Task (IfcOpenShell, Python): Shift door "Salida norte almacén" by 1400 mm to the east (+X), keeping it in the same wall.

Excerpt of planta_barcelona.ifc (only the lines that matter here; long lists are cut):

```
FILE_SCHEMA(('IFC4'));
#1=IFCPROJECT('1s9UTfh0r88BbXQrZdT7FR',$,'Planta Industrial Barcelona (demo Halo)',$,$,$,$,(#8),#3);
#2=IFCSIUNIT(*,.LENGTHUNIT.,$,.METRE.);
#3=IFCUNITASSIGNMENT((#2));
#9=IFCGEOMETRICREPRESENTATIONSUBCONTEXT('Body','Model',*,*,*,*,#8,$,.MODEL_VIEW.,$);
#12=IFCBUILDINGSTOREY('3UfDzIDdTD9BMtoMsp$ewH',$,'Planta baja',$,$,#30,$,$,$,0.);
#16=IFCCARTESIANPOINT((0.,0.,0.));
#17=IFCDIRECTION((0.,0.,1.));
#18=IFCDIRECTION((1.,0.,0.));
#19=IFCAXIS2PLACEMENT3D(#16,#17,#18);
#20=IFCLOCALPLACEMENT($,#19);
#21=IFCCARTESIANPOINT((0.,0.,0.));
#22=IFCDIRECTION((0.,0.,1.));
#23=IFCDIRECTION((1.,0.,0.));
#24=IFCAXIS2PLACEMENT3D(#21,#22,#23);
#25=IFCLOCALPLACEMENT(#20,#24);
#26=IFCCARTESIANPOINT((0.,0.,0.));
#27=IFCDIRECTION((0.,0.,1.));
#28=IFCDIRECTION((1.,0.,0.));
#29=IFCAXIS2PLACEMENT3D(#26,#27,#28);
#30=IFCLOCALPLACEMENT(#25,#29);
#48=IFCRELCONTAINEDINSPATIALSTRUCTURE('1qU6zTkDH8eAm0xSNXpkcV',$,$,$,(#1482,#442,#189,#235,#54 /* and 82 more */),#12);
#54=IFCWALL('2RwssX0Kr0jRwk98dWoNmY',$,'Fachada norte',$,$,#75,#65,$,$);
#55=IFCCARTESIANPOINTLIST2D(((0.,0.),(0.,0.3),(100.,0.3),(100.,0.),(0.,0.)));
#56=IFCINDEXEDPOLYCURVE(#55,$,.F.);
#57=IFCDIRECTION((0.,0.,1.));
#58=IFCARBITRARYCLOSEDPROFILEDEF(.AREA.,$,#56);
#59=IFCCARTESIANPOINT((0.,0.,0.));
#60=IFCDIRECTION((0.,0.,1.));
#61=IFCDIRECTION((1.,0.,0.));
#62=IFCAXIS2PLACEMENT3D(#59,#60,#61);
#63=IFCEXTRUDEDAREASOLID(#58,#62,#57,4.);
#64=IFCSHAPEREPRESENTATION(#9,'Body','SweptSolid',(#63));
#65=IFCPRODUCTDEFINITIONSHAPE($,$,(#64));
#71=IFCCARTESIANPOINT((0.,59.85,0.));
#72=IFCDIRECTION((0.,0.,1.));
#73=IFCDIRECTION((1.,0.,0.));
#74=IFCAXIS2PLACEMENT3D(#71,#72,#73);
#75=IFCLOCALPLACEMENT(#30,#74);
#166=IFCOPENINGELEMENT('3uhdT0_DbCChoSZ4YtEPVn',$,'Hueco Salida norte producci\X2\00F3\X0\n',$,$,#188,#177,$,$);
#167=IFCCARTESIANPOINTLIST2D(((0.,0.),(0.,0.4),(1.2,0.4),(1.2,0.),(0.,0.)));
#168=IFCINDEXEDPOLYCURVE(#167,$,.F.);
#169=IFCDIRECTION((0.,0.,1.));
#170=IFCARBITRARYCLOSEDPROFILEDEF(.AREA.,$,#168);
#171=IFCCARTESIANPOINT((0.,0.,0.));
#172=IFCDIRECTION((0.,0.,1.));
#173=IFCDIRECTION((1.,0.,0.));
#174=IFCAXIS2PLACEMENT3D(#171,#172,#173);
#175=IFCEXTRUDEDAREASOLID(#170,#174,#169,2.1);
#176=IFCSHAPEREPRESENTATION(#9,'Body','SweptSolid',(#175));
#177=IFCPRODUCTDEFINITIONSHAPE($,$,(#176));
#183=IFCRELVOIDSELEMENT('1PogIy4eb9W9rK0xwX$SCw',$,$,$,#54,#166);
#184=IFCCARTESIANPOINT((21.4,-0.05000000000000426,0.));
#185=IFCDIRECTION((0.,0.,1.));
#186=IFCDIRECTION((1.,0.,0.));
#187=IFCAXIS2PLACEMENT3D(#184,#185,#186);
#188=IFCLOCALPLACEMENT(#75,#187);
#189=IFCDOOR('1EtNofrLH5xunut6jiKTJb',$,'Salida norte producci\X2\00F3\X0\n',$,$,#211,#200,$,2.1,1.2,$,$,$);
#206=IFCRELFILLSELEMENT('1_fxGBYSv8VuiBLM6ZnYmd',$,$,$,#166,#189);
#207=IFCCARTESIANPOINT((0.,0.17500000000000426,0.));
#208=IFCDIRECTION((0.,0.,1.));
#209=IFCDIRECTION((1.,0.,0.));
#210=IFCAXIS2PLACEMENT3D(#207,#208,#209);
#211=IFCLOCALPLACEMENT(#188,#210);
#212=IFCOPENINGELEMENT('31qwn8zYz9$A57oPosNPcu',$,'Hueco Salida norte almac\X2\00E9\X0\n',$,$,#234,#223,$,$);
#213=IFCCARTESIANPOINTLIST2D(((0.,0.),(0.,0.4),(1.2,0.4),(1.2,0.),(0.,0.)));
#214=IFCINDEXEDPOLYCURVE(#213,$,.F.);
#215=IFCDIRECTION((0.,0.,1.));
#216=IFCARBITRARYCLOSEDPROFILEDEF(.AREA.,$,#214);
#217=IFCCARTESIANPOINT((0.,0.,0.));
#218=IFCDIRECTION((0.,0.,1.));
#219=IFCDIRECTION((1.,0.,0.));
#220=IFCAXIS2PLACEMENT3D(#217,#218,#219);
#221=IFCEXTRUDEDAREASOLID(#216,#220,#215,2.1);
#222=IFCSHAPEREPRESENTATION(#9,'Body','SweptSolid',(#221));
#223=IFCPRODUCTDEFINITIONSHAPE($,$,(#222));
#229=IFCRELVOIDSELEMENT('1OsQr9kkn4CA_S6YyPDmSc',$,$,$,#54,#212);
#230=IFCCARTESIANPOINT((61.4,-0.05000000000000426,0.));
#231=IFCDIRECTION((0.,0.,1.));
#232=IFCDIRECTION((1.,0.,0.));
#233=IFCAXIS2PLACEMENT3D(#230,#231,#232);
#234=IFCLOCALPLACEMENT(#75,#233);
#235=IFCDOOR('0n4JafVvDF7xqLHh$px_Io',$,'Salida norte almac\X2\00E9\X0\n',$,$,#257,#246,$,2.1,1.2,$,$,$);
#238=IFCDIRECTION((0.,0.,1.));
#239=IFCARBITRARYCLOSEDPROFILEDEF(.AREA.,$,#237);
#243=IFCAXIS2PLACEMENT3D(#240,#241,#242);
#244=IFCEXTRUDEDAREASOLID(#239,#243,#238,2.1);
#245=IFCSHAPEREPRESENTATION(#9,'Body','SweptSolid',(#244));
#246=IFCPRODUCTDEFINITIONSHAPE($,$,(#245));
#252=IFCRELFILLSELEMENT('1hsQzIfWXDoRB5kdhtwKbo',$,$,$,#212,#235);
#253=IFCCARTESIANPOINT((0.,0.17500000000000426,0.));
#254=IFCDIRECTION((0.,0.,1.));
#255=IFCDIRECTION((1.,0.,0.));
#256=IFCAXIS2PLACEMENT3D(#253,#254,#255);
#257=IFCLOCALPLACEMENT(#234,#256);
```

```python
import ifcopenshell
import ifcopenshell.api.geometry
import ifcopenshell.util.placement
import ifcopenshell.util.unit

model = ifcopenshell.open("planta_barcelona.ifc")
unit_scale = ifcopenshell.util.unit.calculate_unit_scale(model)

door = model.by_guid("0n4JafVvDF7xqLHh$px_Io")
opening = door.FillsVoids[0].RelatingOpeningElement
wall = opening.VoidsElements[0].RelatingBuildingElement

wall_matrix = ifcopenshell.util.placement.get_local_placement(wall.ObjectPlacement)
shift = wall_matrix[:3, 0] * 1.4 / unit_scale
before = ifcopenshell.util.placement.get_local_placement(door.ObjectPlacement)[:3, 3].copy()

# The door is placed relative to its opening, so it follows when the opening moves.
matrix = ifcopenshell.util.placement.get_local_placement(opening.ObjectPlacement)
matrix[:3, 3] += shift
ifcopenshell.api.geometry.edit_object_placement(
    model, product=opening, matrix=matrix, is_si=False, should_transform_children=True
)

after = ifcopenshell.util.placement.get_local_placement(door.ObjectPlacement)[:3, 3]
print("door moved by", (after - before).round(3) + 0.0)

model.write("planta_barcelona_updated.ifc")
```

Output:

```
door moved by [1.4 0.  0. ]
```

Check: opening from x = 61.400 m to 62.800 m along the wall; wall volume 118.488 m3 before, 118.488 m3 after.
